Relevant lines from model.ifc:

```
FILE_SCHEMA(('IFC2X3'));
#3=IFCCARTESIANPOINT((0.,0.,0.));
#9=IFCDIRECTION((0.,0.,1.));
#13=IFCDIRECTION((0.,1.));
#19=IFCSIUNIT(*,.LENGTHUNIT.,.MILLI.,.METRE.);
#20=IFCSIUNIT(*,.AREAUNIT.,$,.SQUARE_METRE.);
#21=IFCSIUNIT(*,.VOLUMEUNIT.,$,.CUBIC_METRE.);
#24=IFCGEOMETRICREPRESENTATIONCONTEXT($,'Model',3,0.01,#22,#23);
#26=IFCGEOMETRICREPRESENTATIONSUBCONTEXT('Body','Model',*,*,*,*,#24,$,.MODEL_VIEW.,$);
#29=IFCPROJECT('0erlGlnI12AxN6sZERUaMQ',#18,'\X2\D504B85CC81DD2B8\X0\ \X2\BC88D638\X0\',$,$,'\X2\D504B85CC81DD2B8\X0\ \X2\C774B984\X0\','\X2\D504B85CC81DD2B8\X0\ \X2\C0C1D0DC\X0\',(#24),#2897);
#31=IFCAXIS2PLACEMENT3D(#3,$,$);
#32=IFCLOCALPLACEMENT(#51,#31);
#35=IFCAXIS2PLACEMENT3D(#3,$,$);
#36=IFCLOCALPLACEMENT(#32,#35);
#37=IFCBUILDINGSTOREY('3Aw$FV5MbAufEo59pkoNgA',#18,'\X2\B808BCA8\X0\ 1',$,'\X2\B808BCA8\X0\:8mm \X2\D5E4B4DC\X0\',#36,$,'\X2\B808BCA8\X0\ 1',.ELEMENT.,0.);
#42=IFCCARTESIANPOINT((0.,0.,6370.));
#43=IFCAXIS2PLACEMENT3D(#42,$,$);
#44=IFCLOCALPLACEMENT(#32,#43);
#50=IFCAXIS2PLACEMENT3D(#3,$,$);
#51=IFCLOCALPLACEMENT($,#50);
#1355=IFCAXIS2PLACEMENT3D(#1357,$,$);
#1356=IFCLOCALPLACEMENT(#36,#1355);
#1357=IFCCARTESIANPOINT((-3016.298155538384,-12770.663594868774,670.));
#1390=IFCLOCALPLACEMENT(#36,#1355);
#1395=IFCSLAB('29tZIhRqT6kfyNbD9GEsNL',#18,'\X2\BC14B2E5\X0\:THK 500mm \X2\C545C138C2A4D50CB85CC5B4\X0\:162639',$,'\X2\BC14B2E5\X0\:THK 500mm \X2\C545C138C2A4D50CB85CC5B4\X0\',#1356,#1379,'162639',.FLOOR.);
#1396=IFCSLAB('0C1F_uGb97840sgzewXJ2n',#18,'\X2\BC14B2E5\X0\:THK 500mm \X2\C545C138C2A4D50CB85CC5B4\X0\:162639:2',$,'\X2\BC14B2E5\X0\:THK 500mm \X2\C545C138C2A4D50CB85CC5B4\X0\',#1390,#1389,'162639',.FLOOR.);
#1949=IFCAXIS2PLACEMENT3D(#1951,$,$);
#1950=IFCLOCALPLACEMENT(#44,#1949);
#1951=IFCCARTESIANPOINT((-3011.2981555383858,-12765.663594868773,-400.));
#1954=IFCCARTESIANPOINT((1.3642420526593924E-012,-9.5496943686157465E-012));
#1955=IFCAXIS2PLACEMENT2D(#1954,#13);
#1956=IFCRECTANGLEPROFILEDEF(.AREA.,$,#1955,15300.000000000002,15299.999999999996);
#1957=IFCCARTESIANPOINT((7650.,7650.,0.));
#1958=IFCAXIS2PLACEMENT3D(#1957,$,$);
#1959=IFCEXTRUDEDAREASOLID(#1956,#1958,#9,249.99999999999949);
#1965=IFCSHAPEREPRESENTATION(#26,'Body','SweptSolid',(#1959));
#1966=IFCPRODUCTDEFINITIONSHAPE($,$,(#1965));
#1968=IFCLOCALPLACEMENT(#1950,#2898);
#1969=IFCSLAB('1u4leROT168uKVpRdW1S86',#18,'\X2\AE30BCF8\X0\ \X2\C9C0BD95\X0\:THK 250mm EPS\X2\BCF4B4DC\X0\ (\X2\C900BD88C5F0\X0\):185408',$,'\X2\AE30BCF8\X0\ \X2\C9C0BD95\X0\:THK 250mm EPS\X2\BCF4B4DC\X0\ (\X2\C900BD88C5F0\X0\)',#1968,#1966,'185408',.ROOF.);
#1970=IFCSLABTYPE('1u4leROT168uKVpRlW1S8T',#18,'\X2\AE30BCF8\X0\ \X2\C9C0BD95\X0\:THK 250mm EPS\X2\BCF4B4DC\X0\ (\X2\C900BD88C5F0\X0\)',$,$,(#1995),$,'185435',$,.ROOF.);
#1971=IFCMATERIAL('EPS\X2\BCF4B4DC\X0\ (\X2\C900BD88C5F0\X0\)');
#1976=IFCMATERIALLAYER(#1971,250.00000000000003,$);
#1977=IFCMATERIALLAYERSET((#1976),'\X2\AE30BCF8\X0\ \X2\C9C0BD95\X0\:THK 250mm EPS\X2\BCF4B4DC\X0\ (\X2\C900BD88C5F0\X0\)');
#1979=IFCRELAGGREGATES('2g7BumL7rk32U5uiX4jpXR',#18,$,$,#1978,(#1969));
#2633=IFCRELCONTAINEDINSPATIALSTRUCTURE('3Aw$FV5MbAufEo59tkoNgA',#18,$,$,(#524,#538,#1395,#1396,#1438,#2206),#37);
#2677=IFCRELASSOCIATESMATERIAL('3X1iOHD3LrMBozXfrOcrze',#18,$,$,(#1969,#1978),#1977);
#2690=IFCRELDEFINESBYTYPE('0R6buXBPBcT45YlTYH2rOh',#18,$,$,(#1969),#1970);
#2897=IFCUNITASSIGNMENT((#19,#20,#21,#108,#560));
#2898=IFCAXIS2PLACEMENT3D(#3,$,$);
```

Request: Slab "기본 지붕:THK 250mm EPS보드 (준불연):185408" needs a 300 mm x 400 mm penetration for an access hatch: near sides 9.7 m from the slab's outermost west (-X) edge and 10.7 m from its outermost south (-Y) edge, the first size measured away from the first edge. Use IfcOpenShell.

```python
import numpy as np
import ifcopenshell
import ifcopenshell.api.feature
import ifcopenshell.api.geometry
import ifcopenshell.api.root
import ifcopenshell.geom
import ifcopenshell.util.placement
import ifcopenshell.util.representation
import ifcopenshell.util.shape
import ifcopenshell.util.unit

model = ifcopenshell.open("model.ifc")
unit_scale = ifcopenshell.util.unit.calculate_unit_scale(model)
settings = ifcopenshell.geom.settings()


def volume(element):
    """Net volume in cubic metres, openings subtracted."""
    shape = ifcopenshell.geom.create_shape(settings, element)
    return ifcopenshell.util.shape.get_volume(shape.geometry)


slab = model.by_guid("1u4leROT168uKVpRdW1S86")
before = volume(slab)

# Extent in the slab's own axes, in metres. The edges named are its -X and -Y sides.
slab_shape = ifcopenshell.geom.create_shape(settings, slab)
vertices = ifcopenshell.util.shape.get_vertices(slab_shape.geometry)
x_min, y_min, bottom = vertices.min(axis=0)
top = vertices[:, 2].max()

opening = ifcopenshell.api.root.create_entity(model, ifc_class="IfcOpeningElement", name="Access hatch opening")
context = ifcopenshell.util.representation.get_context(model, "Model", "Body", "MODEL_VIEW")
width, depth = 0.3, 0.4
outline = [(0.0, 0.0), (width, 0.0), (width, depth), (0.0, depth), (0.0, 0.0)]
# Overshoot both faces by 50 mm so the cut is clean.
shape = ifcopenshell.api.geometry.add_slab_representation(
    model, context=context, depth=top - bottom + 0.1, polyline=outline
)
ifcopenshell.api.geometry.assign_representation(model, product=opening, representation=shape)

matrix = ifcopenshell.util.placement.get_local_placement(slab.ObjectPlacement)
matrix[:, 3] = matrix @ np.append(np.array([x_min + 9.7, y_min + 10.7, bottom - 0.05]) / unit_scale, 1.0)
ifcopenshell.api.geometry.edit_object_placement(model, product=opening, matrix=matrix, is_si=False)
ifcopenshell.api.feature.add_feature(model, feature=opening, element=slab)

after = volume(slab)

print(f"slab volume {before:.3f} -> {after:.3f} m3")

model.write("model-out.ifc")
```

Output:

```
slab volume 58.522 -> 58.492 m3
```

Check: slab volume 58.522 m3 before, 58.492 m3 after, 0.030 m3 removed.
